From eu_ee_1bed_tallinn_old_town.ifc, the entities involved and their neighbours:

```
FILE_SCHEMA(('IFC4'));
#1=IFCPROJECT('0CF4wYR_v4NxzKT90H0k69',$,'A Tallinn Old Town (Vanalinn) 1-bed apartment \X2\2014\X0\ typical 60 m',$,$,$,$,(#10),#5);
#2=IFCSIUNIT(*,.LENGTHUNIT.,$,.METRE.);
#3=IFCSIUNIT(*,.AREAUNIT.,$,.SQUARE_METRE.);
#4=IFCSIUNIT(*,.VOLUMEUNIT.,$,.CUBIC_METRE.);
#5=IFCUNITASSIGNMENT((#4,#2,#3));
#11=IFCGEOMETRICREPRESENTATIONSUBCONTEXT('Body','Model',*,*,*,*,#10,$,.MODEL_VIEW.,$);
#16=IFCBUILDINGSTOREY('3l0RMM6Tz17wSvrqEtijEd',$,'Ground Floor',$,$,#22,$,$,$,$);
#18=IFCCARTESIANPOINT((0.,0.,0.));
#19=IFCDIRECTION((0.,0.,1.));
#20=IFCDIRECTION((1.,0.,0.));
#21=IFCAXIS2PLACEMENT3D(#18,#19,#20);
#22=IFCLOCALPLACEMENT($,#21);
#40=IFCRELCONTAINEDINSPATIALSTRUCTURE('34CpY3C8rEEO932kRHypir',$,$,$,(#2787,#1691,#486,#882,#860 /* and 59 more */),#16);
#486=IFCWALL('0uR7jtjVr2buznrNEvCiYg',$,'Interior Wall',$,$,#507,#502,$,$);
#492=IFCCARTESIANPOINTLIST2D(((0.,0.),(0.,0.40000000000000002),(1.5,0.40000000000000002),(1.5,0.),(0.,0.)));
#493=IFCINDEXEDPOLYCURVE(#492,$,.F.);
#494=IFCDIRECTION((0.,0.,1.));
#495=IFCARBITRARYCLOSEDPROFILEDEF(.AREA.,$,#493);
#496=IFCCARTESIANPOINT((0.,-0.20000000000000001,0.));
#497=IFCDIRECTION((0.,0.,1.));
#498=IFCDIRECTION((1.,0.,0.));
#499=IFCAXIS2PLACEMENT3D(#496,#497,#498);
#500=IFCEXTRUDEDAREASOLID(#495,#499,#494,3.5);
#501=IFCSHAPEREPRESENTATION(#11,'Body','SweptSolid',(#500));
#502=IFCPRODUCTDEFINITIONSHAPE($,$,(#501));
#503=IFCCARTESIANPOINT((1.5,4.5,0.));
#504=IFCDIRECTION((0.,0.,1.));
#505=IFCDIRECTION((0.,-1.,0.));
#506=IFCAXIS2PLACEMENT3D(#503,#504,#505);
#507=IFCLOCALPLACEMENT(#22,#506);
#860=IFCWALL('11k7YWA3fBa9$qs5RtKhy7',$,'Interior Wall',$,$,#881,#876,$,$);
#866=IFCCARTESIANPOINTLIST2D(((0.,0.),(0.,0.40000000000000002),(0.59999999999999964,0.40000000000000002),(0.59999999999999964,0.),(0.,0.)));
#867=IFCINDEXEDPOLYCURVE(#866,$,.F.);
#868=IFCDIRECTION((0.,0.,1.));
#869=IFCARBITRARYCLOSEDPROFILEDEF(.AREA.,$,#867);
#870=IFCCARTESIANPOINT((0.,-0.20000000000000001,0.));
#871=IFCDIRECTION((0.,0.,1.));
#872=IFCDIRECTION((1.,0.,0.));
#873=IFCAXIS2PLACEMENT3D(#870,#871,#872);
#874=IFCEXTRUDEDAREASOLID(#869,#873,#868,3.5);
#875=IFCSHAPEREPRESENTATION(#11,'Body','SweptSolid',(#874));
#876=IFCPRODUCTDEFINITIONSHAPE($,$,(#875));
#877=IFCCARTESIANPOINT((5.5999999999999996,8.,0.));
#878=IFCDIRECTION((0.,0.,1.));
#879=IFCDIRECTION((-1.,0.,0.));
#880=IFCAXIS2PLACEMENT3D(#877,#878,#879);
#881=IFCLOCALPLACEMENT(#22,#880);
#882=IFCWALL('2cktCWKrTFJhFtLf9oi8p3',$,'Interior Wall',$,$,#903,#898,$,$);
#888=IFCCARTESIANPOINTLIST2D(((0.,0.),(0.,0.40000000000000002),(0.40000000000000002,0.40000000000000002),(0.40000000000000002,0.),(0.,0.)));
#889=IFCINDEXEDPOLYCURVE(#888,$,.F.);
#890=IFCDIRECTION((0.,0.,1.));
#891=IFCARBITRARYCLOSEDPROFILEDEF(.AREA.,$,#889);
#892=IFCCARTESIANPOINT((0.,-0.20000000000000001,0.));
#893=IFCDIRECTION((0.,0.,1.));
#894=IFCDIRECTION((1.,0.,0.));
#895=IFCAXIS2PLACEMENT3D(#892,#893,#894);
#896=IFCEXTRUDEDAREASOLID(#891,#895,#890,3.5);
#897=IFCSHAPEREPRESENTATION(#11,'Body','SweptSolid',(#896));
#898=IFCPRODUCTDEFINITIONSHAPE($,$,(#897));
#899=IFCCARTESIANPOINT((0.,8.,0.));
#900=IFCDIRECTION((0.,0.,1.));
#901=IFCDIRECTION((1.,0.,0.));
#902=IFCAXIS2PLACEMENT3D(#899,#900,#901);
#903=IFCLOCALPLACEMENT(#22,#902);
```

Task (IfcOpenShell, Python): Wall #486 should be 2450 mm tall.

```python
import ifcopenshell
import ifcopenshell.geom
import ifcopenshell.util.representation
import ifcopenshell.util.shape

model = ifcopenshell.open("eu_ee_1bed_tallinn_old_town.ifc")
settings = ifcopenshell.geom.settings()


def volume(element):
    """Net volume in cubic metres, openings subtracted."""
    shape = ifcopenshell.geom.create_shape(settings, element)
    return ifcopenshell.util.shape.get_volume(shape.geometry)


wall = model.by_guid("0uR7jtjVr2buznrNEvCiYg")
before = volume(wall)

body = ifcopenshell.util.representation.get_representation(wall, "Model", "Body")
solid = body.Items[0]
old_height = solid.Depth
solid.Depth = 2.45
after = volume(wall)

print(f"height {old_height:g} -> {solid.Depth:g}, volume {before:.3f} -> {after:.3f} m3")

model.write("eu_ee_1bed_tallinn_old_town_updated.ifc")
```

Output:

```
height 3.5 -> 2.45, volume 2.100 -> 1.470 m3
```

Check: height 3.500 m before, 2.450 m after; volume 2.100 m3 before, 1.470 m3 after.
